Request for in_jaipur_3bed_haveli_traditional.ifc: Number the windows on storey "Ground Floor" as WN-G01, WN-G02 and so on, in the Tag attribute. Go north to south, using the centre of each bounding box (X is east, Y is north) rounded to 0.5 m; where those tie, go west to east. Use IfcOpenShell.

First a look at what the model holds.

```python
import ifcopenshell
import ifcopenshell.util.element
import ifcopenshell.util.placement

model = ifcopenshell.open("in_jaipur_3bed_haveli_traditional.ifc")
print(model.schema)
storey = next(s for s in model.by_type("IfcBuildingStorey") if s.Name == "Ground Floor")
windows = [e for e in ifcopenshell.util.element.get_decomposition(storey) if e.is_a("IfcWindow")]
for e in sorted(windows, key=lambda e: e.id()):
    origin = ifcopenshell.util.placement.get_local_placement(e.ObjectPlacement)[:3, 3]
    print(e.id(), e.Tag, e.Name, origin.round(2) + 0.0, sep=" | ")
```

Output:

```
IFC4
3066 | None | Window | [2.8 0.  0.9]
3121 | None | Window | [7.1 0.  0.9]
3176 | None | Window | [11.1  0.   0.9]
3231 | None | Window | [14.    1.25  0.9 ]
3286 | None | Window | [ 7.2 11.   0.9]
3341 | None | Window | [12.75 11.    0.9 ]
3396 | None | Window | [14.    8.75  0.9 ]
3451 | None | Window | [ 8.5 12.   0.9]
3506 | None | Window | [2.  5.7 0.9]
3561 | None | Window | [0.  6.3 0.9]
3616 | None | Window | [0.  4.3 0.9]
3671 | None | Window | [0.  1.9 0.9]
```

```python
import ifcopenshell
import ifcopenshell.geom
import ifcopenshell.util.element
import ifcopenshell.util.shape

model = ifcopenshell.open("in_jaipur_3bed_haveli_traditional.ifc")
settings = ifcopenshell.geom.settings()
settings.set("use-world-coords", True)


def centre(element):
    shape = ifcopenshell.geom.create_shape(settings, element)
    return ifcopenshell.util.shape.get_bbox_centroid(shape.geometry)


storey = next(s for s in model.by_type("IfcBuildingStorey") if s.Name == "Ground Floor")
windows = [e for e in ifcopenshell.util.element.get_decomposition(storey) if e.is_a("IfcWindow")]

# Insertion points can sit at a corner or the storey origin, so sort by the geometry (in metres).
centres = {e: centre(e) for e in windows}
windows.sort(key=lambda e: (-round(centres[e][1] / 0.5), centres[e][0]))

for i, e in enumerate(windows, start=1):
    number = f"WN-G{i:02d}"
    e.Tag = number
    print(e.id(), number)

model.write("in_jaipur_3bed_haveli_traditional_rev.ifc")
```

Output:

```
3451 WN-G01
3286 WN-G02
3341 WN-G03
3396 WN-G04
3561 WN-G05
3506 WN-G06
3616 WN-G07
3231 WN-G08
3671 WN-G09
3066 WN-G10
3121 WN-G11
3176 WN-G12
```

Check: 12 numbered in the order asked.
